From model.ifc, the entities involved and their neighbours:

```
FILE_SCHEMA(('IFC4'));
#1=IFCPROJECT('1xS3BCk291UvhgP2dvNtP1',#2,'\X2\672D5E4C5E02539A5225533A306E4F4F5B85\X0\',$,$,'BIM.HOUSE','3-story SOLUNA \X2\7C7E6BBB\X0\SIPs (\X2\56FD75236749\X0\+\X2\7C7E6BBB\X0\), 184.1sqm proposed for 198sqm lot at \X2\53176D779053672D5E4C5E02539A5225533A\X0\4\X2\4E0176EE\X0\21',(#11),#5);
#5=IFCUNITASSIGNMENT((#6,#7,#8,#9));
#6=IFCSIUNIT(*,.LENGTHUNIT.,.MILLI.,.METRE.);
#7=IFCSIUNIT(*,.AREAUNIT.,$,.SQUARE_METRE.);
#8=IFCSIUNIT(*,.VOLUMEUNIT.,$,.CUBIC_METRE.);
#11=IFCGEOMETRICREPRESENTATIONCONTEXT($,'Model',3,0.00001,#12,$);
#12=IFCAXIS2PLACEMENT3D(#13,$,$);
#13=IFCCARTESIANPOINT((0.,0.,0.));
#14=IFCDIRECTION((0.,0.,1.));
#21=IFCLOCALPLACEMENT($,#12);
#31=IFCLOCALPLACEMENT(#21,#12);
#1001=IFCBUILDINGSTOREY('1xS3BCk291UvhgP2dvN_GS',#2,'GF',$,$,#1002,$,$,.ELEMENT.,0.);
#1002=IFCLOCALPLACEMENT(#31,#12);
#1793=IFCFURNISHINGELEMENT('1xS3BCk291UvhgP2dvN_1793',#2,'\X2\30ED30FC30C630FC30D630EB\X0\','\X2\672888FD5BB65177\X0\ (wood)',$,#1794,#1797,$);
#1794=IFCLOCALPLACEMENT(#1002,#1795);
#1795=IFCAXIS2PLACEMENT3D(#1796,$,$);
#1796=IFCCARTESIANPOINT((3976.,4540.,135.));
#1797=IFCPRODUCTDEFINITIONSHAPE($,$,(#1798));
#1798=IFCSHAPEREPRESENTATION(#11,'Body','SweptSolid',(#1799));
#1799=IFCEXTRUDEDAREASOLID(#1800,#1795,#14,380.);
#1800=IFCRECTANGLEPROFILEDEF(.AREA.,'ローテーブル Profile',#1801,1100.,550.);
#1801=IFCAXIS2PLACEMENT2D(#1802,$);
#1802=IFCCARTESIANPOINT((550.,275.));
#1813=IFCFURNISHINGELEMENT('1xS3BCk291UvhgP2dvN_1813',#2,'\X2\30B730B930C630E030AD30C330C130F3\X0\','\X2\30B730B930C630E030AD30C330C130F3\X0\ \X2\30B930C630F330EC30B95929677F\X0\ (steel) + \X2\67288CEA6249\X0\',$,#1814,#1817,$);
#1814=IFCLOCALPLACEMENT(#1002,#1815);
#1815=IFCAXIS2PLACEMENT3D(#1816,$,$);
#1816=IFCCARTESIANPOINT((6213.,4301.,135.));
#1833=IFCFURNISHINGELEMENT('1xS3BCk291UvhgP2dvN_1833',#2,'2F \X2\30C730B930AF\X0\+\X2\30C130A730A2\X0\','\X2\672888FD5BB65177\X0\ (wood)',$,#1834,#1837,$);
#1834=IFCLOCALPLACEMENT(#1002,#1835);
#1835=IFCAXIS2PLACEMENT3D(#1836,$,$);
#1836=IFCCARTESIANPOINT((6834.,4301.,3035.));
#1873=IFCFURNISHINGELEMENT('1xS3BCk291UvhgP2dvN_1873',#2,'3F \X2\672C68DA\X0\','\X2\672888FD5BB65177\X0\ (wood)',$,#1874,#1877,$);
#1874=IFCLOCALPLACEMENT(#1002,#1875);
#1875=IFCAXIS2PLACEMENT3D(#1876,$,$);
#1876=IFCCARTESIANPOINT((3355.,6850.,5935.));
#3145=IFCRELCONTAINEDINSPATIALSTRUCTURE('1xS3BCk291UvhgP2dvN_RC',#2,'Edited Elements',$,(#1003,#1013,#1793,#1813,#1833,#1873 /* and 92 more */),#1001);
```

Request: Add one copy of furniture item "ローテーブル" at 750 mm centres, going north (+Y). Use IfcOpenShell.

```python
import numpy as np
import ifcopenshell
import ifcopenshell.api.geometry
import ifcopenshell.api.root
import ifcopenshell.util.element
import ifcopenshell.util.placement
import ifcopenshell.util.unit

model = ifcopenshell.open("model.ifc")
unit_scale = ifcopenshell.util.unit.calculate_unit_scale(model)


def reuse_history(source, copy):
    """copy_class also copies each property set's owner history, people and application; keep the originals."""
    for rel in copy.IsDefinedBy:
        if rel.is_a("IfcRelDefinesByProperties") and (history := rel.RelatingPropertyDefinition.OwnerHistory):
            rel.RelatingPropertyDefinition.OwnerHistory = source.OwnerHistory
            ifcopenshell.util.element.remove_deep2(model, history)


source = model.by_guid("1xS3BCk291UvhgP2dvN_1793")
base = ifcopenshell.util.placement.get_local_placement(source.ObjectPlacement)
step = np.array([0.0, 1.0, 0.0]) * 0.75 / unit_scale

for i in range(1, 2):
    copy = ifcopenshell.api.root.copy_class(model, product=source)
    copy.Representation = ifcopenshell.util.element.copy_deep(
        model, source.Representation, exclude=["IfcGeometricRepresentationContext", "IfcRepresentationMap"]
    )
    reuse_history(source, copy)
    matrix = base.copy()
    matrix[:3, 3] += i * step
    print("added at", matrix[:3, 3].round(3) + 0.0)
    ifcopenshell.api.geometry.edit_object_placement(model, product=copy, matrix=matrix, is_si=False)

model.write("model_v2.ifc")
```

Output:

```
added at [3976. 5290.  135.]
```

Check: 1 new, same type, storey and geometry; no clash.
